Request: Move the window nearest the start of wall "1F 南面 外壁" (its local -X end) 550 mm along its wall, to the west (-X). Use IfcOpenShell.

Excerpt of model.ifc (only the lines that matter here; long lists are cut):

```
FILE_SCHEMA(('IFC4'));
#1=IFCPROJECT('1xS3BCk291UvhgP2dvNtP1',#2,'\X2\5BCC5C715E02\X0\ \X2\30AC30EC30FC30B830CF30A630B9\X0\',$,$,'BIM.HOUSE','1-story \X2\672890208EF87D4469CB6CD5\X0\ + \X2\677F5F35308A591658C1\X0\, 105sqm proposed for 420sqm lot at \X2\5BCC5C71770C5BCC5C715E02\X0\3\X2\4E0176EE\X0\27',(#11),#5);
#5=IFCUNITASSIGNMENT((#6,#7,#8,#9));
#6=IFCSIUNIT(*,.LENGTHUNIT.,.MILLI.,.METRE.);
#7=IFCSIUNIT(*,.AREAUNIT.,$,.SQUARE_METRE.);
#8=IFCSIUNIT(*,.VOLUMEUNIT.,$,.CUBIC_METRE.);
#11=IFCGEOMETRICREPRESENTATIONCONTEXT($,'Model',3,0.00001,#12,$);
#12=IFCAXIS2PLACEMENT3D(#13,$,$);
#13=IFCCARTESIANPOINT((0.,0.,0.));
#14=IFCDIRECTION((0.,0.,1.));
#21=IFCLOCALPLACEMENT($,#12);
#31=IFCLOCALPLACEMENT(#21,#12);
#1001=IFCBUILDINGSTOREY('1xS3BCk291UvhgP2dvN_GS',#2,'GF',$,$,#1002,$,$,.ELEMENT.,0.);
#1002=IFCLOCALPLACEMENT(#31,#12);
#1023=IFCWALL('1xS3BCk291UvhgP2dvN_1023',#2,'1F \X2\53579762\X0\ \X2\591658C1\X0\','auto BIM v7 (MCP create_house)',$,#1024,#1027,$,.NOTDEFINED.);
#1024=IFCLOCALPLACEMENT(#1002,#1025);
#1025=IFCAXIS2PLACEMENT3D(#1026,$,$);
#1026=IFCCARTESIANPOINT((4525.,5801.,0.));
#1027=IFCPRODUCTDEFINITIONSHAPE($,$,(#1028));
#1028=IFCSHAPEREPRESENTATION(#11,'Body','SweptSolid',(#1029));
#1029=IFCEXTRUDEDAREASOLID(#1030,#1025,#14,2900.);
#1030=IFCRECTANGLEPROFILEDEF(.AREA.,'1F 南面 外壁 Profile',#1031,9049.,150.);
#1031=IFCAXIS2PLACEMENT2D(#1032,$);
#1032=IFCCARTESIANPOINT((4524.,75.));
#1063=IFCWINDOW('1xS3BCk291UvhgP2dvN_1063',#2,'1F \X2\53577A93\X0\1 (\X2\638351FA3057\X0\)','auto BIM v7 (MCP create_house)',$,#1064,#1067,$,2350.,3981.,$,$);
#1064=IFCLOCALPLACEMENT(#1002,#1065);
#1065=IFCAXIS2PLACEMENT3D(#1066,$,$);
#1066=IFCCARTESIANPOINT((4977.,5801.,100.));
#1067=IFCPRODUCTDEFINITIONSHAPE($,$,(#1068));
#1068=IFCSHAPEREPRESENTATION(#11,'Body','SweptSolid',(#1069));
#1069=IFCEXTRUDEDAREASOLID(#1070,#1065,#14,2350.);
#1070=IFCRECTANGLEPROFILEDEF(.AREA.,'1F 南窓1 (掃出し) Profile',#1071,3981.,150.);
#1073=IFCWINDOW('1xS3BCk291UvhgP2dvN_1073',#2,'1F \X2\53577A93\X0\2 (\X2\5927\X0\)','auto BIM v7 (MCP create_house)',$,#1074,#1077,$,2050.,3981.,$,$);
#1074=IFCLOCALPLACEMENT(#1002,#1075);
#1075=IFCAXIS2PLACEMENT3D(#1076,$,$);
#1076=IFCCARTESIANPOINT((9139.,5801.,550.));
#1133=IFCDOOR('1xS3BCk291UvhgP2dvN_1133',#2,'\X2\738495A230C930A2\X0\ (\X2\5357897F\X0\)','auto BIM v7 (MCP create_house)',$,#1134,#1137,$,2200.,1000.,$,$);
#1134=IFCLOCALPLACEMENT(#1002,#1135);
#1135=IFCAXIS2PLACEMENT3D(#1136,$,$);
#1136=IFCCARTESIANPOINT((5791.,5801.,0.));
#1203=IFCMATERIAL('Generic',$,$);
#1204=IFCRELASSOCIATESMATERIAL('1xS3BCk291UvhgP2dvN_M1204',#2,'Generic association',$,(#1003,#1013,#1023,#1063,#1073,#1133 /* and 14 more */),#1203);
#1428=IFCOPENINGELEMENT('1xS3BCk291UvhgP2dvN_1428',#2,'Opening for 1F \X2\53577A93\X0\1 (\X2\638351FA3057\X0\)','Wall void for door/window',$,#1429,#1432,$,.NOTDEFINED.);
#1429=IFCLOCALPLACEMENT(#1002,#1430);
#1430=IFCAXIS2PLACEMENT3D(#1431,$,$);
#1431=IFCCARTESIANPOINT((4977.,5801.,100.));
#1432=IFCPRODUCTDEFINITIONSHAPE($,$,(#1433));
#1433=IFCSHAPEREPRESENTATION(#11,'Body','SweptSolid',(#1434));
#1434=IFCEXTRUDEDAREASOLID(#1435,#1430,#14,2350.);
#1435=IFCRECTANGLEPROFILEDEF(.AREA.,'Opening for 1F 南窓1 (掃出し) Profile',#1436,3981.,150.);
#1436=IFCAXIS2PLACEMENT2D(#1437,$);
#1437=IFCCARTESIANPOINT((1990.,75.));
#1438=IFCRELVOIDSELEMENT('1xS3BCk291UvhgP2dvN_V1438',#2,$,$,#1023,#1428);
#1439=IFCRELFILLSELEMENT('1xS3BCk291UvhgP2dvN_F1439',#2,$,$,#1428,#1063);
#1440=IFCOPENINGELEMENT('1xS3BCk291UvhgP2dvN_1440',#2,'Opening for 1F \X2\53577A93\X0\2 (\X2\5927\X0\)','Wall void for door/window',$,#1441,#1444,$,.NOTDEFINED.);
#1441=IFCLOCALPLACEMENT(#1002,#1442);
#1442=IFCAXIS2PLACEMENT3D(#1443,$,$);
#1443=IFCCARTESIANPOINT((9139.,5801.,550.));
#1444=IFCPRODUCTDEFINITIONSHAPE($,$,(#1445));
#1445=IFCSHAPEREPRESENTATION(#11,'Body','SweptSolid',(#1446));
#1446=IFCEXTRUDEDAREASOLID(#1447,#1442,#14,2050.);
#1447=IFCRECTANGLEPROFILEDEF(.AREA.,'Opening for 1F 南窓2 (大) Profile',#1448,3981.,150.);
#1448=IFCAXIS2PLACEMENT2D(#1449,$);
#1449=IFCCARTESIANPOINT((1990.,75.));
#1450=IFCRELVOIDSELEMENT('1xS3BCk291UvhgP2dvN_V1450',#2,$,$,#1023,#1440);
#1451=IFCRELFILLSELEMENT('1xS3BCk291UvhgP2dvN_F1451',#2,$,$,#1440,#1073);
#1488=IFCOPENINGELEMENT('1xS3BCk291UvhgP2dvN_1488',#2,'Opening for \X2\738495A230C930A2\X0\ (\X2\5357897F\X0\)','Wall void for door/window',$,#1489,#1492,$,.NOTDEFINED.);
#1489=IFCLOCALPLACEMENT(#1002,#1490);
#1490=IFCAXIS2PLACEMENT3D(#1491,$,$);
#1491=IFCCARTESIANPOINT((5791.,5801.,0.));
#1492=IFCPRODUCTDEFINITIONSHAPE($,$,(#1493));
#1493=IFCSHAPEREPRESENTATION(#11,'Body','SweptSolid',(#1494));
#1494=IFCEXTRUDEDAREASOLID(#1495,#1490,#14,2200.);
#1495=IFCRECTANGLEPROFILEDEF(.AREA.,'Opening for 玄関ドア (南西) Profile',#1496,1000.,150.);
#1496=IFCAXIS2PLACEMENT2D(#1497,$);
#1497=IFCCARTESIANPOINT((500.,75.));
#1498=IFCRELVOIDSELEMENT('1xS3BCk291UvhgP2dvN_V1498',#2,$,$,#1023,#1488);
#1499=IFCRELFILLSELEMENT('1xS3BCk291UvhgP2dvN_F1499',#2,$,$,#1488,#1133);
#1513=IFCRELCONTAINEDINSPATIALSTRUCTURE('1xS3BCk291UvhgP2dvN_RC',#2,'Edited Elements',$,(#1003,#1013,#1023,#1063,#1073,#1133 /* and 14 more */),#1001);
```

```python
import ifcopenshell
import ifcopenshell.api.geometry
import ifcopenshell.util.placement

model = ifcopenshell.open("model.ifc")

window = model.by_guid("1xS3BCk291UvhgP2dvN_1063")
opening = window.FillsVoids[0].RelatingOpeningElement
wall = opening.VoidsElements[0].RelatingBuildingElement

wall_matrix = ifcopenshell.util.placement.get_local_placement(wall.ObjectPlacement)
shift = wall_matrix[:3, 0] * -550.0
before = ifcopenshell.util.placement.get_local_placement(window.ObjectPlacement)[:3, 3].copy()

# The window is not placed relative to its opening, so move both.
for product in (opening, window):
    matrix = ifcopenshell.util.placement.get_local_placement(product.ObjectPlacement)
    matrix[:3, 3] += shift
    ifcopenshell.api.geometry.edit_object_placement(model, product=product, matrix=matrix, is_si=False)

after = ifcopenshell.util.placement.get_local_placement(window.ObjectPlacement)[:3, 3]
print("window moved by", (after - before).round(3) + 0.0)

model.write("model-out.ifc")
```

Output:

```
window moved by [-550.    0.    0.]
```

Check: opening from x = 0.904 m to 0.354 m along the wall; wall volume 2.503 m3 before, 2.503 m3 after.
